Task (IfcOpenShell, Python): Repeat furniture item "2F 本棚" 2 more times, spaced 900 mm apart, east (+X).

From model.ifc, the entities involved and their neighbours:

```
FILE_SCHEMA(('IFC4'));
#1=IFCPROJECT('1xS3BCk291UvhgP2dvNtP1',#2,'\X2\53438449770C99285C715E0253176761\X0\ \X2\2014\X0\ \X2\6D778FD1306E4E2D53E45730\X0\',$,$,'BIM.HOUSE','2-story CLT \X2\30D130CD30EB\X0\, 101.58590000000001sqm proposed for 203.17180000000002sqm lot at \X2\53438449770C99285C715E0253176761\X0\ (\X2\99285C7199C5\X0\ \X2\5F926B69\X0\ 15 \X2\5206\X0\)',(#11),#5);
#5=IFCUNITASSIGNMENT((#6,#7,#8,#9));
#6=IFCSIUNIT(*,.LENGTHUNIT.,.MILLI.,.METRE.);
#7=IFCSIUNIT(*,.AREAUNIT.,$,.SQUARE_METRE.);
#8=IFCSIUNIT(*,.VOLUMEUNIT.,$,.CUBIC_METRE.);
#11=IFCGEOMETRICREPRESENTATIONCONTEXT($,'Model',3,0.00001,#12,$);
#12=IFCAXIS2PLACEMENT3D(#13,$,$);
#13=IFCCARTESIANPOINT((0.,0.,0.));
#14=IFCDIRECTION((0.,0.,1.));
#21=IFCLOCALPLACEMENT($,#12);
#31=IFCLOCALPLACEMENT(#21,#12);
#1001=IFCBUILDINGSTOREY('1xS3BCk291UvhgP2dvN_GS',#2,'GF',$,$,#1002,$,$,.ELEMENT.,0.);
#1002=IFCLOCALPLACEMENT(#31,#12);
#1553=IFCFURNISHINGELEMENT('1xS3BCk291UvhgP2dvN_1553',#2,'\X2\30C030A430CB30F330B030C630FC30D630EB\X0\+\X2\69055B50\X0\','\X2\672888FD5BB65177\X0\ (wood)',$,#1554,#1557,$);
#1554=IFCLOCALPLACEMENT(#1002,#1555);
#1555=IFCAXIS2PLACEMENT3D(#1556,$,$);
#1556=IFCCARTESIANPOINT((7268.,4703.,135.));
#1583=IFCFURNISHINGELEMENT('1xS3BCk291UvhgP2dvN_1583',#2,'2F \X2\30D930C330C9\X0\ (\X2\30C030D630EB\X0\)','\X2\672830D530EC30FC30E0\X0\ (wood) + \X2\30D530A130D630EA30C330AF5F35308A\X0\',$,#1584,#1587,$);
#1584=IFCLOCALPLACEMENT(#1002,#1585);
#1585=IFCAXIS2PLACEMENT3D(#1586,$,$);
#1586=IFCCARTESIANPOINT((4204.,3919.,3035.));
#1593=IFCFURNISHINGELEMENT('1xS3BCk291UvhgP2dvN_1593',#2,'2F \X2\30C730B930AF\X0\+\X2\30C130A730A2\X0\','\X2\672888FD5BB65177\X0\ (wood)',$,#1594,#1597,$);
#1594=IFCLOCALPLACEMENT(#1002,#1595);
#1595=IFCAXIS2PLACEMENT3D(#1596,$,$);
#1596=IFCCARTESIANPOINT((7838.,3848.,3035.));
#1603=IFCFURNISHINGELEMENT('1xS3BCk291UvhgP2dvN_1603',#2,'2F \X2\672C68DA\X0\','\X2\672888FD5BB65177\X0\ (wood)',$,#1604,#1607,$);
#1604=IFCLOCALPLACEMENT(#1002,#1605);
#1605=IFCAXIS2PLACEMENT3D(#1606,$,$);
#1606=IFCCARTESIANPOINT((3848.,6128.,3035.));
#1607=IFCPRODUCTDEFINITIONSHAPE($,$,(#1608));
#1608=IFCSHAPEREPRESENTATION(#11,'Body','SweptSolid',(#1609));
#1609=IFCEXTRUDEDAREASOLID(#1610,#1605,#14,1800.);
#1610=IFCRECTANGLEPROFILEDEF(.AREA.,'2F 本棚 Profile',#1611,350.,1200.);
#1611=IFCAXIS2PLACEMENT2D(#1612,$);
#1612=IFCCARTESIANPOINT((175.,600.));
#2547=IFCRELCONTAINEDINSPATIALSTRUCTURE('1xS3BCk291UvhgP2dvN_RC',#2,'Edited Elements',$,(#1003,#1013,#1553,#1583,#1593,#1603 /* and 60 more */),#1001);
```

```python
import numpy as np
import ifcopenshell
import ifcopenshell.api.geometry
import ifcopenshell.api.root
import ifcopenshell.util.element
import ifcopenshell.util.placement

model = ifcopenshell.open("model.ifc")


def reuse_history(source, copy):
    """copy_class also copies each property set's owner history, people and application; keep the originals."""
    for rel in copy.IsDefinedBy:
        if rel.is_a("IfcRelDefinesByProperties") and (history := rel.RelatingPropertyDefinition.OwnerHistory):
            rel.RelatingPropertyDefinition.OwnerHistory = source.OwnerHistory
            ifcopenshell.util.element.remove_deep2(model, history)


source = model.by_guid("1xS3BCk291UvhgP2dvN_1603")
base = ifcopenshell.util.placement.get_local_placement(source.ObjectPlacement)
step = np.array([1.0, 0.0, 0.0]) * 900.0

for i in range(1, 3):
    copy = ifcopenshell.api.root.copy_class(model, product=source)
    copy.Representation = ifcopenshell.util.element.copy_deep(
        model, source.Representation, exclude=["IfcGeometricRepresentationContext", "IfcRepresentationMap"]
    )
    reuse_history(source, copy)
    matrix = base.copy()
    matrix[:3, 3] += i * step
    print("added at", matrix[:3, 3].round(3) + 0.0)
    ifcopenshell.api.geometry.edit_object_placement(model, product=copy, matrix=matrix, is_si=False)

model.write("model-out.ifc")
```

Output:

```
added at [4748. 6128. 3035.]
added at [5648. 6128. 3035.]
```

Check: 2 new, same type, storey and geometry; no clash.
